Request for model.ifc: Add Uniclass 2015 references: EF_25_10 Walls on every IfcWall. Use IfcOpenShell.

First a look at what the model holds.

```python
import ifcopenshell

model = ifcopenshell.open("model.ifc")
print(model.schema)
print("classifications:", [c.Name for c in model.by_type("IfcClassification")])
for ifc_class in ("IfcDoor", "IfcRoof", "IfcStair", "IfcWall", "IfcWindow"):
    print(ifc_class, len(model.by_type(ifc_class)))
```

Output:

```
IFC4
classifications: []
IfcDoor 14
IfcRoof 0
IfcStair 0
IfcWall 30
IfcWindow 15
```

```python
import ifcopenshell
import ifcopenshell.api.classification

model = ifcopenshell.open("model.ifc")

system = ifcopenshell.api.classification.add_classification(model, classification="Uniclass 2015")

codes = {
    "IfcWall": ("EF_25_10", "Walls"),
}
for ifc_class, (code, name) in codes.items():
    products = model.by_type(ifc_class)
    ifcopenshell.api.classification.add_reference(
        model, products=products, classification=system, identification=code, name=name
    )
    print(code, len(products))

model.write("model_updated.ifc")
```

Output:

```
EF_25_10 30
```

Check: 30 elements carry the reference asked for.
